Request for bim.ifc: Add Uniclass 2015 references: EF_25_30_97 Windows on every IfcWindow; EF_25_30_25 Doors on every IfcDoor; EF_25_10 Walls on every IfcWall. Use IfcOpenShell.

First a look at what the model holds.

```python
import ifcopenshell

model = ifcopenshell.open("bim.ifc")
print(model.schema)
print("classifications:", [c.Name for c in model.by_type("IfcClassification")])
for ifc_class in ("IfcDoor", "IfcRoof", "IfcStair", "IfcWall", "IfcWindow"):
    print(ifc_class, len(model.by_type(ifc_class)))
```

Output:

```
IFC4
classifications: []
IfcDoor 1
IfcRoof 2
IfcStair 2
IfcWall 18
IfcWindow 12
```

```python
import ifcopenshell
import ifcopenshell.api.classification

model = ifcopenshell.open("bim.ifc")

system = ifcopenshell.api.classification.add_classification(model, classification="Uniclass 2015")

codes = {
    "IfcWindow": ("EF_25_30_97", "Windows"),
    "IfcDoor": ("EF_25_30_25", "Doors"),
    "IfcWall": ("EF_25_10", "Walls"),
}
for ifc_class, (code, name) in codes.items():
    products = model.by_type(ifc_class)
    ifcopenshell.api.classification.add_reference(
        model, products=products, classification=system, identification=code, name=name
    )
    print(code, len(products))

model.write("bim_edited.ifc")
```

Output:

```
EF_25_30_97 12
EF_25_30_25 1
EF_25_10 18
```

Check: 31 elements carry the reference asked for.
